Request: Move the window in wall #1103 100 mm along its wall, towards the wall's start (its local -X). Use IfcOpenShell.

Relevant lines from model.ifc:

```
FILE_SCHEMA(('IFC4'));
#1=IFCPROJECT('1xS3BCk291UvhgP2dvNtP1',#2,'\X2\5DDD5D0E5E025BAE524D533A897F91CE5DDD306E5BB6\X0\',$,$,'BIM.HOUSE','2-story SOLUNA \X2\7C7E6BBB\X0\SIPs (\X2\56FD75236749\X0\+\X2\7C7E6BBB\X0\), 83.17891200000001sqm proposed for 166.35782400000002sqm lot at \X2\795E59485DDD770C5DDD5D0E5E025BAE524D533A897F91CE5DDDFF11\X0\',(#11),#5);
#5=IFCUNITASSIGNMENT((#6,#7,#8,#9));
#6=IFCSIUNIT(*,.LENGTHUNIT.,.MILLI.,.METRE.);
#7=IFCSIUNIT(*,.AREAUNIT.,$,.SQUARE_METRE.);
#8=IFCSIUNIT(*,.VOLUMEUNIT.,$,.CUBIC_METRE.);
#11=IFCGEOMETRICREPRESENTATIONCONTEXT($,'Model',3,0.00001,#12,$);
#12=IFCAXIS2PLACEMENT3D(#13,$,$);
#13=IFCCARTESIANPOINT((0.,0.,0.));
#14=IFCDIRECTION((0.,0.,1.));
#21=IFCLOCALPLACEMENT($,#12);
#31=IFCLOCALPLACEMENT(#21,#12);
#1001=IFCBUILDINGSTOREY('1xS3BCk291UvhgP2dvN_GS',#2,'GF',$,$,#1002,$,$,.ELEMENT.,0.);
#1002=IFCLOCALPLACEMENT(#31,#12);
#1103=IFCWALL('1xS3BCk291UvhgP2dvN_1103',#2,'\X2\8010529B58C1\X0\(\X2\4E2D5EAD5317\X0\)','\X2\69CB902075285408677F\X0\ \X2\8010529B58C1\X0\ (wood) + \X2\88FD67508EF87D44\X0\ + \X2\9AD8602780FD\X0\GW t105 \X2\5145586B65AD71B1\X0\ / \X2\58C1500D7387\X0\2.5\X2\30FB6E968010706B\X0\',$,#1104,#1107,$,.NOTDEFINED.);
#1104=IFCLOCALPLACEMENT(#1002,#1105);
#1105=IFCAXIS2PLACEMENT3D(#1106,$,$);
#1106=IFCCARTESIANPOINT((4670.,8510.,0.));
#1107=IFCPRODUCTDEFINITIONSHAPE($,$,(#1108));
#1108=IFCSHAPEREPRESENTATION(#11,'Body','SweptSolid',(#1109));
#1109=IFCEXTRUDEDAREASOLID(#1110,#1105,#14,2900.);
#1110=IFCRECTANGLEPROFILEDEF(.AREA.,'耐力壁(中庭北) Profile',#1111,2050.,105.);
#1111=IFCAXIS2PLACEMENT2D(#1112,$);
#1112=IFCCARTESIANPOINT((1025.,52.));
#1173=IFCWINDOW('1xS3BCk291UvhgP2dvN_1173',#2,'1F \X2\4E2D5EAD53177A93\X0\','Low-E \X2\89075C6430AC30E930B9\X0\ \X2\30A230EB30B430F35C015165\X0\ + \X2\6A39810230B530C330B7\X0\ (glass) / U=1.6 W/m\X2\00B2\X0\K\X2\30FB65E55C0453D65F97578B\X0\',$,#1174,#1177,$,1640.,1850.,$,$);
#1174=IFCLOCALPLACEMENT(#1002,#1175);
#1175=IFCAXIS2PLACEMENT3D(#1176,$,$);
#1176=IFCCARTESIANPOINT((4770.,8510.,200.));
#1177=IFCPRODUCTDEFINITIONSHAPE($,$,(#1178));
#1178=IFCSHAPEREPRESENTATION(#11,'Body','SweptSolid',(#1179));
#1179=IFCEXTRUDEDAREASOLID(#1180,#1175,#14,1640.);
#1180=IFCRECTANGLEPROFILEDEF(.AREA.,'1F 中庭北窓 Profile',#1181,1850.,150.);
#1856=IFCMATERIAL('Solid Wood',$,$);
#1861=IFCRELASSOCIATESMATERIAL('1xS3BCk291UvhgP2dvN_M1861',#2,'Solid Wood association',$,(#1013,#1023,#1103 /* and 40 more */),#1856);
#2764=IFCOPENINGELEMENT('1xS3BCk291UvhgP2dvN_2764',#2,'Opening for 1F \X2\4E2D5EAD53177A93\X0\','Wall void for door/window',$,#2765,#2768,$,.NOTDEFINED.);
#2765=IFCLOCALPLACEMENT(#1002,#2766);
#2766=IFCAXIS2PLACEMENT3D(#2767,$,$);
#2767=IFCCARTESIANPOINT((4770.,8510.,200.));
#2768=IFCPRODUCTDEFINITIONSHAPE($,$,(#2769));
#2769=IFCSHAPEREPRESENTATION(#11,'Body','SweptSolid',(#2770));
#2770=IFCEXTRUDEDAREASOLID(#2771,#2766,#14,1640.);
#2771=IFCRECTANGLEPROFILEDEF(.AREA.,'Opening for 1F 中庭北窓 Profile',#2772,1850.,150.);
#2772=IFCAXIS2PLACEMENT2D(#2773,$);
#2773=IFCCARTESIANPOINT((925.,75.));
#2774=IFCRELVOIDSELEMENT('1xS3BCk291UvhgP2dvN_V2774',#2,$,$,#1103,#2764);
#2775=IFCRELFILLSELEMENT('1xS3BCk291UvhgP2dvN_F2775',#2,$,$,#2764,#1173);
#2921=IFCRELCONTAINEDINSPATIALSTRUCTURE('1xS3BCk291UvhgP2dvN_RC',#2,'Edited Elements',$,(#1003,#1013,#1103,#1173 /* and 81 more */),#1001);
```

```python
import ifcopenshell
import ifcopenshell.api.geometry
import ifcopenshell.util.placement
import ifcopenshell.util.unit

model = ifcopenshell.open("model.ifc")
unit_scale = ifcopenshell.util.unit.calculate_unit_scale(model)

window = model.by_id(1173)
opening = window.FillsVoids[0].RelatingOpeningElement
wall = opening.VoidsElements[0].RelatingBuildingElement

wall_matrix = ifcopenshell.util.placement.get_local_placement(wall.ObjectPlacement)
shift = wall_matrix[:3, 0] * -0.1 / unit_scale
before = ifcopenshell.util.placement.get_local_placement(window.ObjectPlacement)[:3, 3].copy()

# The window is not placed relative to its opening, so move both.
for product in (opening, window):
    matrix = ifcopenshell.util.placement.get_local_placement(product.ObjectPlacement)
    matrix[:3, 3] += shift
    ifcopenshell.api.geometry.edit_object_placement(model, product=product, matrix=matrix, is_si=False)

after = ifcopenshell.util.placement.get_local_placement(window.ObjectPlacement)[:3, 3]
print("window moved by", (after - before).round(3) + 0.0)

model.write("model_v2.ifc")
```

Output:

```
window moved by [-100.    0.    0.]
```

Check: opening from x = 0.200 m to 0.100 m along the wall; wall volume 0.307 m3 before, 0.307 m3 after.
